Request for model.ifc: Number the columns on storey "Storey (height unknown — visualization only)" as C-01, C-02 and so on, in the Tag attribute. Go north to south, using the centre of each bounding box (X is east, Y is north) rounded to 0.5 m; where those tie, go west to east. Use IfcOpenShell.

First a look at what the model holds.

```python
import ifcopenshell
import ifcopenshell.util.element
import ifcopenshell.util.placement

model = ifcopenshell.open("model.ifc")
print(model.schema)
storey = next(s for s in model.by_type("IfcBuildingStorey") if s.Name == "Storey (height unknown — visualization only)")
columns = [e for e in ifcopenshell.util.element.get_decomposition(storey) if e.is_a("IfcColumn")]
for e in sorted(columns, key=lambda e: e.id()):
    origin = ifcopenshell.util.placement.get_local_placement(e.ObjectPlacement)[:3, 3]
    print(e.id(), e.Tag, e.Name, origin.round(2) + 0.0, sep=" | ")
```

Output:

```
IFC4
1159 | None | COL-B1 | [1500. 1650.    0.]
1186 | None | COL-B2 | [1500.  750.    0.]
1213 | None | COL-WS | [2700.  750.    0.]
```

```python
import ifcopenshell
import ifcopenshell.geom
import ifcopenshell.util.element
import ifcopenshell.util.shape

model = ifcopenshell.open("model.ifc")
settings = ifcopenshell.geom.settings()
settings.set("use-world-coords", True)


def centre(element):
    shape = ifcopenshell.geom.create_shape(settings, element)
    return ifcopenshell.util.shape.get_bbox_centroid(shape.geometry)


storey = next(s for s in model.by_type("IfcBuildingStorey") if s.Name == "Storey (height unknown — visualization only)")
columns = [e for e in ifcopenshell.util.element.get_decomposition(storey) if e.is_a("IfcColumn")]

# Insertion points can sit at a corner or the storey origin, so sort by the geometry (in metres).
centres = {e: centre(e) for e in columns}
columns.sort(key=lambda e: (-round(centres[e][1] / 0.5), centres[e][0]))

for i, e in enumerate(columns, start=1):
    number = f"C-{i:02d}"
    e.Tag = number
    print(e.id(), number)

model.write("model_rev.ifc")
```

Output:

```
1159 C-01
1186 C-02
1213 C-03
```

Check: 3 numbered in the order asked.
